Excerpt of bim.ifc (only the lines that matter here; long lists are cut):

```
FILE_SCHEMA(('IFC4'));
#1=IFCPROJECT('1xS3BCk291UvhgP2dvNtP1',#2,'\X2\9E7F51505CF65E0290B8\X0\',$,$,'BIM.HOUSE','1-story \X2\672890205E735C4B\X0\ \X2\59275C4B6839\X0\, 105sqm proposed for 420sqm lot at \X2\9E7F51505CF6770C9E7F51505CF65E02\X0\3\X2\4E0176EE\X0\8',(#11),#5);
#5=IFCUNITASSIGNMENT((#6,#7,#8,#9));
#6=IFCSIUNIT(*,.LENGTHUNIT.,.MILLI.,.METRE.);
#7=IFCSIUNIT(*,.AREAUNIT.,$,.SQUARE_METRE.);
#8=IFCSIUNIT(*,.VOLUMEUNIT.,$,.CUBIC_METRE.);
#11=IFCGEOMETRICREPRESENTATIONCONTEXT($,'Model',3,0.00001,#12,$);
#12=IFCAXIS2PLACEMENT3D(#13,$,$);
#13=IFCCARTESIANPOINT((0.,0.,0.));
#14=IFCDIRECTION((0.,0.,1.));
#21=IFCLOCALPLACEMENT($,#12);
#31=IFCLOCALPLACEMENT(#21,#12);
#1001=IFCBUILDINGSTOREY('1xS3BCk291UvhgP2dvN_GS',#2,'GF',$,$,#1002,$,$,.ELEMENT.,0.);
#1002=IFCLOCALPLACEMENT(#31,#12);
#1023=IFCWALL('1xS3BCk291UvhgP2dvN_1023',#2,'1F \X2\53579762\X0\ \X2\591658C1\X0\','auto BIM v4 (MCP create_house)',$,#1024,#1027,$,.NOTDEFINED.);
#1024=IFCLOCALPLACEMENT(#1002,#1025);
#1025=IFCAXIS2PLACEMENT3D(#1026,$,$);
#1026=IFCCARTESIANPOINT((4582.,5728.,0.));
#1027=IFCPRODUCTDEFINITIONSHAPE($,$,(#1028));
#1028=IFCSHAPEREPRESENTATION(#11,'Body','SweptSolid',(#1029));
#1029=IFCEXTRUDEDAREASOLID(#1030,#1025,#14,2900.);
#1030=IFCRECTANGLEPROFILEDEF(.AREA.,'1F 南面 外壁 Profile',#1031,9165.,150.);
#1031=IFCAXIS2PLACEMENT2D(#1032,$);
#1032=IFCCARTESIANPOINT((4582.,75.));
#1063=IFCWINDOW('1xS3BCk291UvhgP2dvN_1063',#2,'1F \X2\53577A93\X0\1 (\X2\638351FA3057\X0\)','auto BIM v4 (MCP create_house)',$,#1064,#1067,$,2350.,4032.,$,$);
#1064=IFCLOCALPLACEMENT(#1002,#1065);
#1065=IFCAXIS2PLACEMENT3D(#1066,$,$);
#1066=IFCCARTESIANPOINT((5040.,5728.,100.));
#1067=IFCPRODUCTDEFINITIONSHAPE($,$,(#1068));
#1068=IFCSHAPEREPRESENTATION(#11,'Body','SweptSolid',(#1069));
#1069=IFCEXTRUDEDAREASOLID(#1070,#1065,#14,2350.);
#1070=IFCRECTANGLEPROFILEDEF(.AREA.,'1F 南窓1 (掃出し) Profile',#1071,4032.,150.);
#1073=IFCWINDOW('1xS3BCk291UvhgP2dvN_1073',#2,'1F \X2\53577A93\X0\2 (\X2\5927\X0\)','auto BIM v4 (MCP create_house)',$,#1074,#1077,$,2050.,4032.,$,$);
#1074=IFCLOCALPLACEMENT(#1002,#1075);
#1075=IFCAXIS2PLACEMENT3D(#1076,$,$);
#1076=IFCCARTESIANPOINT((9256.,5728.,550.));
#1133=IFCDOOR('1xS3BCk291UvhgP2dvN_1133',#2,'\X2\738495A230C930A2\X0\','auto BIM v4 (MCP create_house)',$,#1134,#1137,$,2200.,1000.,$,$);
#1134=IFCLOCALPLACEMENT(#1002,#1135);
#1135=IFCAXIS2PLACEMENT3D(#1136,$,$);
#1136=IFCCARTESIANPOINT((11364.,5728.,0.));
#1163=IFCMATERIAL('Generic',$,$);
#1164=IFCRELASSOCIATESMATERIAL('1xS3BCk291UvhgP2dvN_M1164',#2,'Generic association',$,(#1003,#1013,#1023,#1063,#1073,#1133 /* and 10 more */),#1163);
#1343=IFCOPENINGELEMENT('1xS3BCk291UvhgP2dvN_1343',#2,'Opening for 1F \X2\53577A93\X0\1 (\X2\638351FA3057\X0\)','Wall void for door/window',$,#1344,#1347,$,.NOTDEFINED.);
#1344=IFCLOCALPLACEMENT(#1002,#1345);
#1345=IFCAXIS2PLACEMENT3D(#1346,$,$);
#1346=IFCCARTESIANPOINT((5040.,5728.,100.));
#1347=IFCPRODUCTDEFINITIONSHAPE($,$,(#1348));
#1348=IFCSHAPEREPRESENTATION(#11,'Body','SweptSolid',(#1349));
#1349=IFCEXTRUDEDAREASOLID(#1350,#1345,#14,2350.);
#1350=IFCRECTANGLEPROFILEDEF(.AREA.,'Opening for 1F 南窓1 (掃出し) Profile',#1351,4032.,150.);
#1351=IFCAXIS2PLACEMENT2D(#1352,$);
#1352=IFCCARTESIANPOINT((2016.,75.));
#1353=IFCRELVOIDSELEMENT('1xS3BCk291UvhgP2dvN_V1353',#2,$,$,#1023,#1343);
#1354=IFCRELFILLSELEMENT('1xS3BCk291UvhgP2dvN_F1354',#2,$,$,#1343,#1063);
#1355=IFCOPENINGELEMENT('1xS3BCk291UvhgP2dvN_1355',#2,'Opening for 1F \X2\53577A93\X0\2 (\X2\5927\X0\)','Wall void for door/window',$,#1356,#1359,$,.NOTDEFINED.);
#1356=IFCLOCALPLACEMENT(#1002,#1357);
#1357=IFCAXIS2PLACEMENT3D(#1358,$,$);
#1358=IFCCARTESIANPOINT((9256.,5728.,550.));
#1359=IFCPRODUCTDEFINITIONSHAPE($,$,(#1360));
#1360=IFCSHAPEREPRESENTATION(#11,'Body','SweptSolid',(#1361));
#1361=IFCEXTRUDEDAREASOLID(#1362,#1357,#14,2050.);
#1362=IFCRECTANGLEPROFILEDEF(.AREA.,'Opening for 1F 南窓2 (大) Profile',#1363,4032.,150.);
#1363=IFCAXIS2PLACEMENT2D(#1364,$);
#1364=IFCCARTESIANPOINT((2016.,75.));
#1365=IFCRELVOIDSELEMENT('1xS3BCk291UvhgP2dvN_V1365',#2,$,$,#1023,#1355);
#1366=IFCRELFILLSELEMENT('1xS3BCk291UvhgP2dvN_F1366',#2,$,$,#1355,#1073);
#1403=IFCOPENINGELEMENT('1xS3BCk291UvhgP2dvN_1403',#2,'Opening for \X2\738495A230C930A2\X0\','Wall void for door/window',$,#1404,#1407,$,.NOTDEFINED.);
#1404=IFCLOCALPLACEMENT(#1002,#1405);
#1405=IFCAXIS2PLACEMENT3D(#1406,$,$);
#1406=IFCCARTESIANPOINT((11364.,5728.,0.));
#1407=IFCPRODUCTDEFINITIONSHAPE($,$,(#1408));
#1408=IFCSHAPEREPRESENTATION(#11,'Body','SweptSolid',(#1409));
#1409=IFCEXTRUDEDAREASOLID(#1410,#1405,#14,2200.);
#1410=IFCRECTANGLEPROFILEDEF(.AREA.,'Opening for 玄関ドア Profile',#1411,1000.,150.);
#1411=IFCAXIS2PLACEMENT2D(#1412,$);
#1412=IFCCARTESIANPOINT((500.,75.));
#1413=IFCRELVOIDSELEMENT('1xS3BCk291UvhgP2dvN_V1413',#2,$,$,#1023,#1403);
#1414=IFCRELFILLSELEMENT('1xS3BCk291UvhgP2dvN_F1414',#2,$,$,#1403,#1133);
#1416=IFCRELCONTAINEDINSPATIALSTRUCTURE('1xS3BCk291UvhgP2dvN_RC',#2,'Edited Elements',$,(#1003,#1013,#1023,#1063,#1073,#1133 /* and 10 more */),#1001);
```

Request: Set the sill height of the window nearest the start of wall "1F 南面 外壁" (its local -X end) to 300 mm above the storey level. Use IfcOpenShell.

```python
import numpy as np
import ifcopenshell
import ifcopenshell.api.geometry
import ifcopenshell.geom
import ifcopenshell.util.element
import ifcopenshell.util.placement
import ifcopenshell.util.shape
import ifcopenshell.util.unit

model = ifcopenshell.open("bim.ifc")
unit_scale = ifcopenshell.util.unit.calculate_unit_scale(model)

window = model.by_id(1063)
opening = window.FillsVoids[0].RelatingOpeningElement
storey = ifcopenshell.util.element.get_container(window, ifc_class="IfcBuildingStorey")
level = ifcopenshell.util.placement.get_local_placement(storey.ObjectPlacement)[2, 3]

# The opening's origin need not be at the sill, so measure its lowest point.
shape = ifcopenshell.geom.create_shape(ifcopenshell.geom.settings(), opening)
bottom = ifcopenshell.util.shape.get_shape_bottom_elevation(shape, shape.geometry) / unit_scale
dz = level + 300.0 - bottom

shift = np.array([0.0, 0.0, dz])
# The window is not placed relative to its opening, so move both.
for product in (opening, window):
    matrix = ifcopenshell.util.placement.get_local_placement(product.ObjectPlacement)
    matrix[:3, 3] += shift
    ifcopenshell.api.geometry.edit_object_placement(model, product=product, matrix=matrix, is_si=False)

print(f"moved by {dz * unit_scale:+.3f} m")

model.write("bim_edited.ifc")
```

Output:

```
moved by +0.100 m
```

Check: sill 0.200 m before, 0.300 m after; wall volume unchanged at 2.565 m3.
